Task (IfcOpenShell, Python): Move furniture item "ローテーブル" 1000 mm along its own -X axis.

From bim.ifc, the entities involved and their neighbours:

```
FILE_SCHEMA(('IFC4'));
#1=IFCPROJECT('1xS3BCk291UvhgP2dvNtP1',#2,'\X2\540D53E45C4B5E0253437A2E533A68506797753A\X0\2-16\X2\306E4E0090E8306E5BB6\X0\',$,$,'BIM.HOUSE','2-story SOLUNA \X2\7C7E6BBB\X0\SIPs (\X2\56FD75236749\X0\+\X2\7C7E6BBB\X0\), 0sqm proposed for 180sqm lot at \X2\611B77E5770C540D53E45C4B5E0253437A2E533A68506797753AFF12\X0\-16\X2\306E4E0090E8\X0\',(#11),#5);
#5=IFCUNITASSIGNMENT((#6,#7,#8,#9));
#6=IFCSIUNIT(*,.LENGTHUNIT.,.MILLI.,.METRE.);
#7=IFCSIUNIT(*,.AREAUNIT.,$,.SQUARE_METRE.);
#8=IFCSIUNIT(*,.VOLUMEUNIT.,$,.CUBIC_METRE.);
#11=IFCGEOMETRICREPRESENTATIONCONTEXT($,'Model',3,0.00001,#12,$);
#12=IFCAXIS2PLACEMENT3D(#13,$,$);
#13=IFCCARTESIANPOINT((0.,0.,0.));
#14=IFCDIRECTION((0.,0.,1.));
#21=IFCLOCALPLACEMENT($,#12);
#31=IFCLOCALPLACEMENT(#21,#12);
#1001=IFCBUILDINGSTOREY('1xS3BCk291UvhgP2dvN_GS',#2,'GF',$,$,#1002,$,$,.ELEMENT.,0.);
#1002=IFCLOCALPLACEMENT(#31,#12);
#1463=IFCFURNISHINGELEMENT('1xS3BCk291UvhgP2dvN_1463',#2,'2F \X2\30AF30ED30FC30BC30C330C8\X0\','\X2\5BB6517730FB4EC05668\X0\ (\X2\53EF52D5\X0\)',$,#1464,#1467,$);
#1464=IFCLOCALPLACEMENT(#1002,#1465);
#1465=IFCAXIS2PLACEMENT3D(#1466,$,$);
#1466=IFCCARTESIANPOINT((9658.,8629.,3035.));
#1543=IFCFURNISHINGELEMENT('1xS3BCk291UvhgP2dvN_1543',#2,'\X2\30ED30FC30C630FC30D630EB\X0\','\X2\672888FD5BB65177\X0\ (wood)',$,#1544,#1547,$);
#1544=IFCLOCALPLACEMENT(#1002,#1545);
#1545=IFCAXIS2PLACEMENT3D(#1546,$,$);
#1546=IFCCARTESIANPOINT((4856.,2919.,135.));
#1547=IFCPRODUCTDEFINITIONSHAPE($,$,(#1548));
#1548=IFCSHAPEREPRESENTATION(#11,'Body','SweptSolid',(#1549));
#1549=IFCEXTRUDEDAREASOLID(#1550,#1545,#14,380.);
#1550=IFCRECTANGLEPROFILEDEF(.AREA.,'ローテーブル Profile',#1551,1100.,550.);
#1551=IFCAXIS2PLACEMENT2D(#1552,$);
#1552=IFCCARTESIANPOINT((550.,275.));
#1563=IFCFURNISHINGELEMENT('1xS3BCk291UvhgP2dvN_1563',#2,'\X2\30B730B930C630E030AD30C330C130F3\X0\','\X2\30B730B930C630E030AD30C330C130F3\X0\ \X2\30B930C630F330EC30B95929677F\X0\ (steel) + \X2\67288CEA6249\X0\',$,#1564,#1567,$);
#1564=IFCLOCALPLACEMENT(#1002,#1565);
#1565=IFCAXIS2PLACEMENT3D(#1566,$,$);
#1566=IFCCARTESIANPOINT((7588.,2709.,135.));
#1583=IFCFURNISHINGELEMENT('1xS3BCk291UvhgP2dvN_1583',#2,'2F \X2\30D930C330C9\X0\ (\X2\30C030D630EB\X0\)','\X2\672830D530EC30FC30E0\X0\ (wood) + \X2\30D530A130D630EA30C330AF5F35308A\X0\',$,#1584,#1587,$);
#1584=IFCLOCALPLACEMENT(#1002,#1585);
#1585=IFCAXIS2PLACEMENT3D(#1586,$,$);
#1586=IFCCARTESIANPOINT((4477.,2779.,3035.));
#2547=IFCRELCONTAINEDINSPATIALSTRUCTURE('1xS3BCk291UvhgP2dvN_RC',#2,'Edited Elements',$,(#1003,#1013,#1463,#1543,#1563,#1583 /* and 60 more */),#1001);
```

```python
import ifcopenshell
import ifcopenshell.api.geometry
import ifcopenshell.util.placement

model = ifcopenshell.open("bim.ifc")

item = model.by_guid("1xS3BCk291UvhgP2dvN_1543")
matrix = ifcopenshell.util.placement.get_local_placement(item.ObjectPlacement)
matrix[:3, 3] -= matrix[:3, 0] * 1000.0
ifcopenshell.api.geometry.edit_object_placement(model, product=item, matrix=matrix, is_si=False)

print(ifcopenshell.util.placement.get_local_placement(item.ObjectPlacement).round(3) + 0.0)

model.write("bim_edited.ifc")
```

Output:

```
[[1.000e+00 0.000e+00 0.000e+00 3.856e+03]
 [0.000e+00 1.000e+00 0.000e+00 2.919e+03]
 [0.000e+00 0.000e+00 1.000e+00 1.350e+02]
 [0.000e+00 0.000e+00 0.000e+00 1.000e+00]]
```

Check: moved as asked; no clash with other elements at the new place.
